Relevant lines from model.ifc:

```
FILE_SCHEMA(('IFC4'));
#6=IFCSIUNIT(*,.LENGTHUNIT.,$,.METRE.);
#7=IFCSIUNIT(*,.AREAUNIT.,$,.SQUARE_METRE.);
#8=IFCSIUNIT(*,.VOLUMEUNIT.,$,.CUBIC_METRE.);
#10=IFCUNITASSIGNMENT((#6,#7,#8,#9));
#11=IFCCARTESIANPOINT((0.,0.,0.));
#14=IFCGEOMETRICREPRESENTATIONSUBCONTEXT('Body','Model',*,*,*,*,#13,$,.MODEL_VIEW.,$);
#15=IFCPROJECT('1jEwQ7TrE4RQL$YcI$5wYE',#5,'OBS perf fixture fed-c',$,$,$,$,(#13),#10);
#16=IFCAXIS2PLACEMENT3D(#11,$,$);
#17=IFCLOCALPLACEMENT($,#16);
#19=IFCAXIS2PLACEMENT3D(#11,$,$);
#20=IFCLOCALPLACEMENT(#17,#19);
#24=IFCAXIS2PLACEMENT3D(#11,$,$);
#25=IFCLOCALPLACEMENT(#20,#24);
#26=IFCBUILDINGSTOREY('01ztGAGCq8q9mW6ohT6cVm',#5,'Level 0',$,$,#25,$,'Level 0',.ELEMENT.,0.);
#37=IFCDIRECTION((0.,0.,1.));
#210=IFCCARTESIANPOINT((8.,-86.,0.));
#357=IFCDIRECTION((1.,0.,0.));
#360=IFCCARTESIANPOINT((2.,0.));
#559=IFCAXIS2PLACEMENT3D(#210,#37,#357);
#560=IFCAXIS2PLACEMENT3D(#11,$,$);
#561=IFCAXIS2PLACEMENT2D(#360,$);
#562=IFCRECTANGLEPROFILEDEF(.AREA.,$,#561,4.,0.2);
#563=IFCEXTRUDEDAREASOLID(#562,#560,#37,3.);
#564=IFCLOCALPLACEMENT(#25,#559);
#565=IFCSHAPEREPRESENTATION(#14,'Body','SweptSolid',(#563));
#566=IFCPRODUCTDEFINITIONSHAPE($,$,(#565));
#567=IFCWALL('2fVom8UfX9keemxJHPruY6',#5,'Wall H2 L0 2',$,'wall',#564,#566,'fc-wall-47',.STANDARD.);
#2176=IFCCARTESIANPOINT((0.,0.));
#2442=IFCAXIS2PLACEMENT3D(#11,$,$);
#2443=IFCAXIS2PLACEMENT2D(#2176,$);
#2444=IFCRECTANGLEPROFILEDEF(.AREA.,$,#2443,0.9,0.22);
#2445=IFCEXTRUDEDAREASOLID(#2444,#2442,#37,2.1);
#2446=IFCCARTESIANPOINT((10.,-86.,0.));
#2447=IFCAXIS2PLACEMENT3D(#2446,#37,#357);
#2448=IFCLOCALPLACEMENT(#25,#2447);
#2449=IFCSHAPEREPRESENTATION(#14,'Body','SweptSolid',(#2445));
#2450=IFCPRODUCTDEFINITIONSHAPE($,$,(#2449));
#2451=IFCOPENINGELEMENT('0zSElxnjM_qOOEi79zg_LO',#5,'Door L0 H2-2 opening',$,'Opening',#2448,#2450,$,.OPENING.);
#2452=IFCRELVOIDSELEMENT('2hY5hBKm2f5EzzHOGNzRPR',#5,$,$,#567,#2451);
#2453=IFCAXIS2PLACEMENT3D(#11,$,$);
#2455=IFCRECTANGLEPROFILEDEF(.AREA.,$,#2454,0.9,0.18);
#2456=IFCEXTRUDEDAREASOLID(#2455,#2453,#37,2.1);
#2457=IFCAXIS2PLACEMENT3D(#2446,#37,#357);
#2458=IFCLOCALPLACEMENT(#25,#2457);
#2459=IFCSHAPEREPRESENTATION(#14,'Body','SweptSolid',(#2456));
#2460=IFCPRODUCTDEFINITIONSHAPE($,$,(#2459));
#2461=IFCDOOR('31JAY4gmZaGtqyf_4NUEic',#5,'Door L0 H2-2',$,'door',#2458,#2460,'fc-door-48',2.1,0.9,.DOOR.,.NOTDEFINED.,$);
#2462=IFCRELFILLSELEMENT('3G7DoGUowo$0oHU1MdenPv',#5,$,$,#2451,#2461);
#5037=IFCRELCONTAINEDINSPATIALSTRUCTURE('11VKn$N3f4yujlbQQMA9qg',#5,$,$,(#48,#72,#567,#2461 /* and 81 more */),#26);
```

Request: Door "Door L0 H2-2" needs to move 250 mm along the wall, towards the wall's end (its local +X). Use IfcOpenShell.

```python
import ifcopenshell
import ifcopenshell.api.geometry
import ifcopenshell.util.placement
import ifcopenshell.util.unit

model = ifcopenshell.open("model.ifc")
unit_scale = ifcopenshell.util.unit.calculate_unit_scale(model)

door = model.by_guid("31JAY4gmZaGtqyf_4NUEic")
opening = door.FillsVoids[0].RelatingOpeningElement
wall = opening.VoidsElements[0].RelatingBuildingElement

wall_matrix = ifcopenshell.util.placement.get_local_placement(wall.ObjectPlacement)
shift = wall_matrix[:3, 0] * 0.25 / unit_scale
before = ifcopenshell.util.placement.get_local_placement(door.ObjectPlacement)[:3, 3].copy()

# The door is not placed relative to its opening, so move both.
for product in (opening, door):
    matrix = ifcopenshell.util.placement.get_local_placement(product.ObjectPlacement)
    matrix[:3, 3] += shift
    ifcopenshell.api.geometry.edit_object_placement(model, product=product, matrix=matrix, is_si=False)

after = ifcopenshell.util.placement.get_local_placement(door.ObjectPlacement)[:3, 3]
print("door moved by", (after - before).round(3) + 0.0)

model.write("model_edited.ifc")
```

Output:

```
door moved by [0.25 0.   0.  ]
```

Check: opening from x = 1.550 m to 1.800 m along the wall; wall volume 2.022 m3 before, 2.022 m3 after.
